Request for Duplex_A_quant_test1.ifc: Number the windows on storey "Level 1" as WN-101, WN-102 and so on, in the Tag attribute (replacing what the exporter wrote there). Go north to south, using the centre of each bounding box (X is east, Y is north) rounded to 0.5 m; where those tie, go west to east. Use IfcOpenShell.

First a look at what the model holds.

```python
import ifcopenshell
import ifcopenshell.util.element
import ifcopenshell.util.placement

model = ifcopenshell.open("Duplex_A_quant_test1.ifc")
print(model.schema)
storey = next(s for s in model.by_type("IfcBuildingStorey") if s.Name == "Level 1")
windows = [e for e in ifcopenshell.util.element.get_decomposition(storey) if e.is_a("IfcWindow")]
for e in sorted(windows, key=lambda e: e.id()):
    origin = ifcopenshell.util.placement.get_local_placement(e.ObjectPlacement)[:3, 3]
    print(e.id(), e.Tag, e.Name, origin.round(2) + 0.0, sep=" | ")
```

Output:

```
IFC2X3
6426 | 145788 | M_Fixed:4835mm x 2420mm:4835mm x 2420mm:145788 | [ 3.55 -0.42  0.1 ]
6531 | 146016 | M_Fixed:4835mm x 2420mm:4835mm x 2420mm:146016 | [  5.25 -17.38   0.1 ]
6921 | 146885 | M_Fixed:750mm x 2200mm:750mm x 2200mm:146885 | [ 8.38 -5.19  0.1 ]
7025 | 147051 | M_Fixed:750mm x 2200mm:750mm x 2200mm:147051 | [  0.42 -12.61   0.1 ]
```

```python
import ifcopenshell
import ifcopenshell.geom
import ifcopenshell.util.element
import ifcopenshell.util.shape

model = ifcopenshell.open("Duplex_A_quant_test1.ifc")
settings = ifcopenshell.geom.settings()
settings.set("use-world-coords", True)


def centre(element):
    shape = ifcopenshell.geom.create_shape(settings, element)
    return ifcopenshell.util.shape.get_bbox_centroid(shape.geometry)


storey = next(s for s in model.by_type("IfcBuildingStorey") if s.Name == "Level 1")
windows = [e for e in ifcopenshell.util.element.get_decomposition(storey) if e.is_a("IfcWindow")]

# Insertion points can sit at a corner or the storey origin, so sort by the geometry (in metres).
centres = {e: centre(e) for e in windows}
windows.sort(key=lambda e: (-round(centres[e][1] / 0.5), centres[e][0]))

for i, e in enumerate(windows, start=1):
    number = f"WN-1{i:02d}"
    e.Tag = number
    print(e.id(), number)

model.write("Duplex_A_quant_test1_v2.ifc")
```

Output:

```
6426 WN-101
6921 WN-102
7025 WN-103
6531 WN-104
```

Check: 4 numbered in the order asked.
